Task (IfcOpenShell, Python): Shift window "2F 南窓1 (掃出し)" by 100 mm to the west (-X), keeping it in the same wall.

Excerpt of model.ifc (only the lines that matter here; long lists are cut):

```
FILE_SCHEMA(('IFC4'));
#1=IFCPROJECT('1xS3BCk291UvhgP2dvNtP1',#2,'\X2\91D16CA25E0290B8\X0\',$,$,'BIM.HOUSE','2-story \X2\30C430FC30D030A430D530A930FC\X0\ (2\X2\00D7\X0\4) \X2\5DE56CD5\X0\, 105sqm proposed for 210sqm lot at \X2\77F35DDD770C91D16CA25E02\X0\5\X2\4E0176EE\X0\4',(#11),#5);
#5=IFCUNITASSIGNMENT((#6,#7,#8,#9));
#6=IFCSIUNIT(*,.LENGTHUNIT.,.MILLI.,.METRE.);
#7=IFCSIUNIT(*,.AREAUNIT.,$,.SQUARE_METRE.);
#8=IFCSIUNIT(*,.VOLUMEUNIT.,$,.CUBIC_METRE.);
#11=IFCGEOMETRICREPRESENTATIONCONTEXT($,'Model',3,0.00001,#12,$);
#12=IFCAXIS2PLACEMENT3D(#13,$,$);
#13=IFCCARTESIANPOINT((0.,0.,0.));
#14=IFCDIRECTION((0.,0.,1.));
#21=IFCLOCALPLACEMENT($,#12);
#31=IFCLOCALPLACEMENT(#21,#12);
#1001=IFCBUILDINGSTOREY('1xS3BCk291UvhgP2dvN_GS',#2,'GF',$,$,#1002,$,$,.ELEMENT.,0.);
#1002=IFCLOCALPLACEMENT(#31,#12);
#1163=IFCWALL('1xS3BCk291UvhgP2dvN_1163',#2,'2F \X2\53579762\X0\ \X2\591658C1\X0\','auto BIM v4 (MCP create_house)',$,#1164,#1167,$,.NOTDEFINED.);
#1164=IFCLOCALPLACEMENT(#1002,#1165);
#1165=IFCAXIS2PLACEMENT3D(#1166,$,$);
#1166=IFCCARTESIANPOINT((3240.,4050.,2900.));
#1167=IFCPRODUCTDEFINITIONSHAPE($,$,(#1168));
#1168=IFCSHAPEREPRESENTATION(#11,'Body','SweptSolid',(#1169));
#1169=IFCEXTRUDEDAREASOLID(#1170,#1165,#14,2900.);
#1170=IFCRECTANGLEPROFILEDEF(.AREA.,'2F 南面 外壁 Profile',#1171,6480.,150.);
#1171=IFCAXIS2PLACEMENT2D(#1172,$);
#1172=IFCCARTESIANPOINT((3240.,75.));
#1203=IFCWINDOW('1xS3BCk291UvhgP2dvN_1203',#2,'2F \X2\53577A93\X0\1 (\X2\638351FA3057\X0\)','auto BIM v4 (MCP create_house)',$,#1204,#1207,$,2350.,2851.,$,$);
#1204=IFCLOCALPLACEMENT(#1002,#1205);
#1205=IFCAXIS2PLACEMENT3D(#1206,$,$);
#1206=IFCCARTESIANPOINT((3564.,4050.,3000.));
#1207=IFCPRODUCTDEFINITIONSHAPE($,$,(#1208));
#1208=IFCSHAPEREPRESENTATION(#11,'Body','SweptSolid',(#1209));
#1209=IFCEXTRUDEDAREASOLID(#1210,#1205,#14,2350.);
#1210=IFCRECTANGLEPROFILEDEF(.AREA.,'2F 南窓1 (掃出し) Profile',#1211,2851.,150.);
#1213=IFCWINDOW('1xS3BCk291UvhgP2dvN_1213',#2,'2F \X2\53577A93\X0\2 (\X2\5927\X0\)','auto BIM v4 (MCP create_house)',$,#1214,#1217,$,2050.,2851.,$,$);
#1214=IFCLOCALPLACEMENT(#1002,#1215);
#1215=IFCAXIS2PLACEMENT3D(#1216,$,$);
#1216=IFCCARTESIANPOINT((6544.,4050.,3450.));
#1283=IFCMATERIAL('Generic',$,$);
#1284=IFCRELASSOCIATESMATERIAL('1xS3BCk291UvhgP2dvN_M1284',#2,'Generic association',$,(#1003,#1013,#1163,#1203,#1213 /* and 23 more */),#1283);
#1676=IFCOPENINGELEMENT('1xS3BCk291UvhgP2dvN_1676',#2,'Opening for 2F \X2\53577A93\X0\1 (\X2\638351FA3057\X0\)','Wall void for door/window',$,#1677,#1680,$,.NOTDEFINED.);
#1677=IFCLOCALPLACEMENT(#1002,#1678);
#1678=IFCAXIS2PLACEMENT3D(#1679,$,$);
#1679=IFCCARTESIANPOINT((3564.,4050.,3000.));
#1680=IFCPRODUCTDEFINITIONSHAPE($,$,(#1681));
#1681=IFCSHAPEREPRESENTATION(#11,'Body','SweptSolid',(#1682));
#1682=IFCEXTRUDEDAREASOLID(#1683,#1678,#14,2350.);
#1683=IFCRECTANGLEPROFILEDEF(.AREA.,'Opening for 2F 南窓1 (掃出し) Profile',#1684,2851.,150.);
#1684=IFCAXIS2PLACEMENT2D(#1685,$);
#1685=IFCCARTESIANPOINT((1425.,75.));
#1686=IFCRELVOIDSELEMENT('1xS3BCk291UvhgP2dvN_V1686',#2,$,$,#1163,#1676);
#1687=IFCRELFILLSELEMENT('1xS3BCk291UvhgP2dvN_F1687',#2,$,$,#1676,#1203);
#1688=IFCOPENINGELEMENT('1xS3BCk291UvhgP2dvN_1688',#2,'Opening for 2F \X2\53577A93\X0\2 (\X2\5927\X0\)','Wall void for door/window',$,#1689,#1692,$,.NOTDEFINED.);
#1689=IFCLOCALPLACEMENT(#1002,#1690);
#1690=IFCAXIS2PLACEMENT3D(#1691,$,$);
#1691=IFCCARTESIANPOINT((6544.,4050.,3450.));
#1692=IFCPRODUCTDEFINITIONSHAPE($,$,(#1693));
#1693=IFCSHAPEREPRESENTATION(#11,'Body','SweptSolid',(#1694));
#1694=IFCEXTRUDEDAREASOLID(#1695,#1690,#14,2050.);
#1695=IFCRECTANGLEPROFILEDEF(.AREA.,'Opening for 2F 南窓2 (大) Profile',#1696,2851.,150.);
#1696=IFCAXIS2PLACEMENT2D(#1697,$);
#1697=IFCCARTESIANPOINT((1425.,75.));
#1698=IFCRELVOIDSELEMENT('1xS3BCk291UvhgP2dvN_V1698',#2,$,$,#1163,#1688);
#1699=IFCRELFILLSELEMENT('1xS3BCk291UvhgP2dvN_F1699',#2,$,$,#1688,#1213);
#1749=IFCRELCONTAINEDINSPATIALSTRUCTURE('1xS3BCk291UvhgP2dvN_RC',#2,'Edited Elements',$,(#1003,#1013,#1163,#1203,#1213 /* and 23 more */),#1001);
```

```python
import ifcopenshell
import ifcopenshell.api.geometry
import ifcopenshell.util.placement
import ifcopenshell.util.unit

model = ifcopenshell.open("model.ifc")
unit_scale = ifcopenshell.util.unit.calculate_unit_scale(model)

window = model.by_guid("1xS3BCk291UvhgP2dvN_1203")
opening = window.FillsVoids[0].RelatingOpeningElement
wall = opening.VoidsElements[0].RelatingBuildingElement

wall_matrix = ifcopenshell.util.placement.get_local_placement(wall.ObjectPlacement)
shift = wall_matrix[:3, 0] * -0.1 / unit_scale
before = ifcopenshell.util.placement.get_local_placement(window.ObjectPlacement)[:3, 3].copy()

# The window is not placed relative to its opening, so move both.
for product in (opening, window):
    matrix = ifcopenshell.util.placement.get_local_placement(product.ObjectPlacement)
    matrix[:3, 3] += shift
    ifcopenshell.api.geometry.edit_object_placement(model, product=product, matrix=matrix, is_si=False)

after = ifcopenshell.util.placement.get_local_placement(window.ObjectPlacement)[:3, 3]
print("window moved by", (after - before).round(3) + 0.0)

model.write("model-out.ifc")
```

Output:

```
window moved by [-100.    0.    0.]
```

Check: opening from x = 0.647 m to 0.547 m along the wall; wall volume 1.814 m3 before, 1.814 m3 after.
